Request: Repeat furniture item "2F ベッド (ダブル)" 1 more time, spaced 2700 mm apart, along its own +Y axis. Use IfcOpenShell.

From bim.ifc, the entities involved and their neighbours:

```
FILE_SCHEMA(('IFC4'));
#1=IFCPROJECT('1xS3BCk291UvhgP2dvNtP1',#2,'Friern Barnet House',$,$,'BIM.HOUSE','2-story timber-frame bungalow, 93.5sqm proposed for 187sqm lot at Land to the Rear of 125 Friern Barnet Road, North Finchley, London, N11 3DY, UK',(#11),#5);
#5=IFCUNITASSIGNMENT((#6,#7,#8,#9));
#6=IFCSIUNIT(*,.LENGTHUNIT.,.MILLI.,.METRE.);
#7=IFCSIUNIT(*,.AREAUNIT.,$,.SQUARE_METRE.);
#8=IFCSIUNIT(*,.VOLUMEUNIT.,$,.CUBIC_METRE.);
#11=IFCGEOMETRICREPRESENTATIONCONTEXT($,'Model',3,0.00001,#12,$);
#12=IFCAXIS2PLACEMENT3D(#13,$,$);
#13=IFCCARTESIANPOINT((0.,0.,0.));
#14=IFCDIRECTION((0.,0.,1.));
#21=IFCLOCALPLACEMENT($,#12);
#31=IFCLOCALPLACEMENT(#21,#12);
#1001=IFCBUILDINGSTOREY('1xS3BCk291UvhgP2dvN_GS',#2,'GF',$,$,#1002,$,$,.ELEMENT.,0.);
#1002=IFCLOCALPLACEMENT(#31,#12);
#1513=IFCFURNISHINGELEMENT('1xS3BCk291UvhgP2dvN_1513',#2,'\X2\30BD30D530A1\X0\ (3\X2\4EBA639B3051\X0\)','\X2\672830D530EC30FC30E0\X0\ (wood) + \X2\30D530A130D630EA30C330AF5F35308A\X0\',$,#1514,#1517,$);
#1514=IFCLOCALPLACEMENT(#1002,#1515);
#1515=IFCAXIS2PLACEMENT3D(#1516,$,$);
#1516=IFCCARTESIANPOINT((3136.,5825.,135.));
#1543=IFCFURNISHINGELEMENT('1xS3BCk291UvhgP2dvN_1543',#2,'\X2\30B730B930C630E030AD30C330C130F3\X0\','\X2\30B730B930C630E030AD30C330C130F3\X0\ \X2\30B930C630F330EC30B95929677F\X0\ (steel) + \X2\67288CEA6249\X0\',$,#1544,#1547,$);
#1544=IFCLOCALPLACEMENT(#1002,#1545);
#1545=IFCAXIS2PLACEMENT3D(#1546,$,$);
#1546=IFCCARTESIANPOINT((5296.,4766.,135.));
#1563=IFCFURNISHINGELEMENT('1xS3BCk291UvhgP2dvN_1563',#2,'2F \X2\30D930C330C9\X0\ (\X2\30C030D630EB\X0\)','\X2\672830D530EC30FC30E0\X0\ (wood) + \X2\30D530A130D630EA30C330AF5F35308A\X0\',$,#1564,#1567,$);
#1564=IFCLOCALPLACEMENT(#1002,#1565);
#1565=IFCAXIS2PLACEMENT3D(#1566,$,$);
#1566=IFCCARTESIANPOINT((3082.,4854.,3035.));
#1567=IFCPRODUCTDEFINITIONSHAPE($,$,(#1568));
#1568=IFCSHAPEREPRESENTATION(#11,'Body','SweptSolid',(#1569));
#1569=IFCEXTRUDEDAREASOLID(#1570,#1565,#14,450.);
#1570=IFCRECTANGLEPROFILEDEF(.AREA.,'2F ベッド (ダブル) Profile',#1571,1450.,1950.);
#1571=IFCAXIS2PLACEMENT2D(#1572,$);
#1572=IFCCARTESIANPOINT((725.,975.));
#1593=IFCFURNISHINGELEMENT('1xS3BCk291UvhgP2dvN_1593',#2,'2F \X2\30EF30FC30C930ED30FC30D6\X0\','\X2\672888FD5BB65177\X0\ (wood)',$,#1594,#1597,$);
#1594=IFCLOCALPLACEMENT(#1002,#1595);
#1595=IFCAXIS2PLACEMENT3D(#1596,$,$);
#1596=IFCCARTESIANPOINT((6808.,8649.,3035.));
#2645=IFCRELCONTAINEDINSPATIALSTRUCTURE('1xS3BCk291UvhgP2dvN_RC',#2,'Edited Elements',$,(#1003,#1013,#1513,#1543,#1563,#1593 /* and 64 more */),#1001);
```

```python
import ifcopenshell
import ifcopenshell.api.geometry
import ifcopenshell.api.root
import ifcopenshell.util.element
import ifcopenshell.util.placement
import ifcopenshell.util.unit

model = ifcopenshell.open("bim.ifc")
unit_scale = ifcopenshell.util.unit.calculate_unit_scale(model)


def reuse_history(source, copy):
    """copy_class also copies each property set's owner history, people and application; keep the originals."""
    for rel in copy.IsDefinedBy:
        if rel.is_a("IfcRelDefinesByProperties") and (history := rel.RelatingPropertyDefinition.OwnerHistory):
            rel.RelatingPropertyDefinition.OwnerHistory = source.OwnerHistory
            ifcopenshell.util.element.remove_deep2(model, history)


source = model.by_guid("1xS3BCk291UvhgP2dvN_1563")
base = ifcopenshell.util.placement.get_local_placement(source.ObjectPlacement)
step = base[:3, 1] * 2.7 / unit_scale

for i in range(1, 2):
    copy = ifcopenshell.api.root.copy_class(model, product=source)
    copy.Representation = ifcopenshell.util.element.copy_deep(
        model, source.Representation, exclude=["IfcGeometricRepresentationContext", "IfcRepresentationMap"]
    )
    reuse_history(source, copy)
    matrix = base.copy()
    matrix[:3, 3] += i * step
    print("added at", matrix[:3, 3].round(3) + 0.0)
    ifcopenshell.api.geometry.edit_object_placement(model, product=copy, matrix=matrix, is_si=False)

model.write("bim_rev.ifc")
```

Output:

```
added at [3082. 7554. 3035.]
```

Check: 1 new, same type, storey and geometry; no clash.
